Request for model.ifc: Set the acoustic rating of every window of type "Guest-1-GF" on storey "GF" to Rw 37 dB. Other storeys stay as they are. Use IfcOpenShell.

First a look at what the model holds.

```python
import ifcopenshell
import ifcopenshell.util.element

model = ifcopenshell.open("model.ifc")
print(model.schema)
storey = next(s for s in model.by_type("IfcBuildingStorey") if s.Name == "GF")
windows = [e for e in ifcopenshell.util.element.get_decomposition(storey) if e.is_a("IfcWindow")]
seen = {}
for e in windows:
    element_type = ifcopenshell.util.element.get_type(e)
    key = (element_type.Name if element_type != e and element_type else None, ifcopenshell.util.element.get_pset(e, "Pset_WindowCommon", "AcousticRating"))
    seen[key] = seen.get(key, 0) + 1
for (name, value), count in sorted(seen.items(), key=str):
    print(count, "x", name, "|", value)
```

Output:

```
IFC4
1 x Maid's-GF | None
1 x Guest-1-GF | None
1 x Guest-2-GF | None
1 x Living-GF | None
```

```python
import ifcopenshell
import ifcopenshell.api.pset
import ifcopenshell.util.element

model = ifcopenshell.open("model.ifc")

storey = next(s for s in model.by_type("IfcBuildingStorey") if s.Name == "GF")
windows = [e for e in ifcopenshell.util.element.get_decomposition(storey) if e.is_a("IfcWindow")]

count = 0
for e in windows:
    element_type = ifcopenshell.util.element.get_type(e)
    if element_type in (None, e) or element_type.Name != "Guest-1-GF":
        continue
    # add_pset returns the element's existing set when there is one.
    pset = ifcopenshell.api.pset.add_pset(model, product=e, name="Pset_WindowCommon")
    ifcopenshell.api.pset.edit_pset(model, pset=pset, properties={"AcousticRating": "Rw 37 dB"})
    count += 1

print(count, "windows updated")

model.write("model-out.ifc")
```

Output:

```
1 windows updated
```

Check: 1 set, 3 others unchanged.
